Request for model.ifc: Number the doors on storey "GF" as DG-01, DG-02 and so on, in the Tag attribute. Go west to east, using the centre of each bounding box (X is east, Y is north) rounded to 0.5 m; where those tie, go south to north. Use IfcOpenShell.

First a look at what the model holds.

```python
import ifcopenshell
import ifcopenshell.util.element
import ifcopenshell.util.placement

model = ifcopenshell.open("model.ifc")
print(model.schema)
storey = next(s for s in model.by_type("IfcBuildingStorey") if s.Name == "GF")
doors = [e for e in ifcopenshell.util.element.get_decomposition(storey) if e.is_a("IfcDoor")]
for e in sorted(doors, key=lambda e: e.id()):
    origin = ifcopenshell.util.placement.get_local_placement(e.ObjectPlacement)[:3, 3]
    print(e.id(), e.Tag, e.Name, origin.round(2) + 0.0, sep=" | ")
```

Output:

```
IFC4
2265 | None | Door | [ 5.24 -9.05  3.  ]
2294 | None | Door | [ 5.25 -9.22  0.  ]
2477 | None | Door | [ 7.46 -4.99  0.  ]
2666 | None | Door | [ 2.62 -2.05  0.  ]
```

```python
import ifcopenshell
import ifcopenshell.geom
import ifcopenshell.util.element
import ifcopenshell.util.shape

model = ifcopenshell.open("model.ifc")
settings = ifcopenshell.geom.settings()
settings.set("use-world-coords", True)


def centre(element):
    shape = ifcopenshell.geom.create_shape(settings, element)
    return ifcopenshell.util.shape.get_bbox_centroid(shape.geometry)


storey = next(s for s in model.by_type("IfcBuildingStorey") if s.Name == "GF")
doors = [e for e in ifcopenshell.util.element.get_decomposition(storey) if e.is_a("IfcDoor")]

# Insertion points can sit at a corner or the storey origin, so sort by the geometry (in metres).
centres = {e: centre(e) for e in doors}
doors.sort(key=lambda e: (round(centres[e][0] / 0.5), centres[e][1]))

for i, e in enumerate(doors, start=1):
    number = f"DG-{i:02d}"
    e.Tag = number
    print(e.id(), number)

model.write("model_rev.ifc")
```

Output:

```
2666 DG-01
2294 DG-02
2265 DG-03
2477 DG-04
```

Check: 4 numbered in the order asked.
